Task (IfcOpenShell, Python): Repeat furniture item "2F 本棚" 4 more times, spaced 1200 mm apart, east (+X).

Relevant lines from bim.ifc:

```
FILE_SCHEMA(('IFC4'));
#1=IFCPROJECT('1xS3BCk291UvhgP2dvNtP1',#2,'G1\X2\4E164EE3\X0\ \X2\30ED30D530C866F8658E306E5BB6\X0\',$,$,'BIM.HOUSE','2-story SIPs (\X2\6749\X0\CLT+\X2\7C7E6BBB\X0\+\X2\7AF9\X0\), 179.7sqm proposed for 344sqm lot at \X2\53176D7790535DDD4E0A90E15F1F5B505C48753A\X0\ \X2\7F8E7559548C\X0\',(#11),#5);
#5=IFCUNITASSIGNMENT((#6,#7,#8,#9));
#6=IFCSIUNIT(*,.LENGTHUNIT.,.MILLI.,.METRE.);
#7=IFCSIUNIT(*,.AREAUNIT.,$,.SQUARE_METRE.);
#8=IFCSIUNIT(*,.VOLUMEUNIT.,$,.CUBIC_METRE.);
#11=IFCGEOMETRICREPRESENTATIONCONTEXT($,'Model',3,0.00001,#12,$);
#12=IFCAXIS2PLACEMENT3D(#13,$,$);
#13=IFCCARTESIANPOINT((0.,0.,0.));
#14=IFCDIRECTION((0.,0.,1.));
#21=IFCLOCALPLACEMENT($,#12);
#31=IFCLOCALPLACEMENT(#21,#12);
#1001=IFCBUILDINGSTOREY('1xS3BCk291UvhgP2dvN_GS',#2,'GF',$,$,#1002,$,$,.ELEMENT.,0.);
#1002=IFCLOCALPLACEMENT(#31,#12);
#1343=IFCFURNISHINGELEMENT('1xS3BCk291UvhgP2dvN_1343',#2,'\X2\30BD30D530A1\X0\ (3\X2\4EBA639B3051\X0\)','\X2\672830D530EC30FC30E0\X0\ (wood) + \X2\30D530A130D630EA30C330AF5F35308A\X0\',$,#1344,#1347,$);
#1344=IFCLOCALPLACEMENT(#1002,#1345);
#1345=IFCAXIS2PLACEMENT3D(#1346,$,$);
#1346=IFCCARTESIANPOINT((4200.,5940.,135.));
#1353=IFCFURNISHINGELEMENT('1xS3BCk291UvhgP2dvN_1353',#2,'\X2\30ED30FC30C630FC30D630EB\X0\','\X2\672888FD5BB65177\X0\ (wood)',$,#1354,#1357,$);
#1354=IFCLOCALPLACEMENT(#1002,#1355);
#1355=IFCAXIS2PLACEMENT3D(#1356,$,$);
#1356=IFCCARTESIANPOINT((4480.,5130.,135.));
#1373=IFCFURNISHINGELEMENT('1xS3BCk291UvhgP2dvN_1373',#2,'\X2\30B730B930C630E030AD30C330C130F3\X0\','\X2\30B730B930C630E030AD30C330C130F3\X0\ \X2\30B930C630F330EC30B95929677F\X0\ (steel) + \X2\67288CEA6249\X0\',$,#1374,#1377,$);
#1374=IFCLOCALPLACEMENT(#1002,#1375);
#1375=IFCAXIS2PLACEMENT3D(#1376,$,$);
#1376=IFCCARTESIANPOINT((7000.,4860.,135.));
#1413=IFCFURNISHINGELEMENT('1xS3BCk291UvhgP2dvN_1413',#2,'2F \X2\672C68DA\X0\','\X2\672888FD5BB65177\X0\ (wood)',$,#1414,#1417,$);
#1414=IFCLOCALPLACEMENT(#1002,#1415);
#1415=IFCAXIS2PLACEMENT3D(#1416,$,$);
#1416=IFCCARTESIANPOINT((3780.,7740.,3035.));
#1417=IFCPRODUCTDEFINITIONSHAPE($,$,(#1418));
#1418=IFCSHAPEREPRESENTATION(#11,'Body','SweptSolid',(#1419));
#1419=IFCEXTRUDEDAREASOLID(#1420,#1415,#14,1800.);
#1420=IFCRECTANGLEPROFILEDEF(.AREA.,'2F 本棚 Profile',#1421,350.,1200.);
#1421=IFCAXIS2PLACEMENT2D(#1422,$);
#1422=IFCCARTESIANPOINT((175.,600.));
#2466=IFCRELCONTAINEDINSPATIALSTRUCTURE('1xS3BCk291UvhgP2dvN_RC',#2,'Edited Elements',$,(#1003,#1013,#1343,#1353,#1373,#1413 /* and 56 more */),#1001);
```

```python
import numpy as np
import ifcopenshell
import ifcopenshell.api.geometry
import ifcopenshell.api.root
import ifcopenshell.util.element
import ifcopenshell.util.placement
import ifcopenshell.util.unit

model = ifcopenshell.open("bim.ifc")
unit_scale = ifcopenshell.util.unit.calculate_unit_scale(model)


def reuse_history(source, copy):
    """copy_class also copies each property set's owner history, people and application; keep the originals."""
    for rel in copy.IsDefinedBy:
        if rel.is_a("IfcRelDefinesByProperties") and (history := rel.RelatingPropertyDefinition.OwnerHistory):
            rel.RelatingPropertyDefinition.OwnerHistory = source.OwnerHistory
            ifcopenshell.util.element.remove_deep2(model, history)


source = model.by_id(1413)
base = ifcopenshell.util.placement.get_local_placement(source.ObjectPlacement)
step = np.array([1.0, 0.0, 0.0]) * 1.2 / unit_scale

for i in range(1, 5):
    copy = ifcopenshell.api.root.copy_class(model, product=source)
    copy.Representation = ifcopenshell.util.element.copy_deep(
        model, source.Representation, exclude=["IfcGeometricRepresentationContext", "IfcRepresentationMap"]
    )
    reuse_history(source, copy)
    matrix = base.copy()
    matrix[:3, 3] += i * step
    print("added at", matrix[:3, 3].round(3) + 0.0)
    ifcopenshell.api.geometry.edit_object_placement(model, product=copy, matrix=matrix, is_si=False)

model.write("bim_v2.ifc")
```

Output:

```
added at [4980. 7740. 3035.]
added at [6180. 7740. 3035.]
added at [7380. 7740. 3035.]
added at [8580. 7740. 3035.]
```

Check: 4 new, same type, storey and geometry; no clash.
